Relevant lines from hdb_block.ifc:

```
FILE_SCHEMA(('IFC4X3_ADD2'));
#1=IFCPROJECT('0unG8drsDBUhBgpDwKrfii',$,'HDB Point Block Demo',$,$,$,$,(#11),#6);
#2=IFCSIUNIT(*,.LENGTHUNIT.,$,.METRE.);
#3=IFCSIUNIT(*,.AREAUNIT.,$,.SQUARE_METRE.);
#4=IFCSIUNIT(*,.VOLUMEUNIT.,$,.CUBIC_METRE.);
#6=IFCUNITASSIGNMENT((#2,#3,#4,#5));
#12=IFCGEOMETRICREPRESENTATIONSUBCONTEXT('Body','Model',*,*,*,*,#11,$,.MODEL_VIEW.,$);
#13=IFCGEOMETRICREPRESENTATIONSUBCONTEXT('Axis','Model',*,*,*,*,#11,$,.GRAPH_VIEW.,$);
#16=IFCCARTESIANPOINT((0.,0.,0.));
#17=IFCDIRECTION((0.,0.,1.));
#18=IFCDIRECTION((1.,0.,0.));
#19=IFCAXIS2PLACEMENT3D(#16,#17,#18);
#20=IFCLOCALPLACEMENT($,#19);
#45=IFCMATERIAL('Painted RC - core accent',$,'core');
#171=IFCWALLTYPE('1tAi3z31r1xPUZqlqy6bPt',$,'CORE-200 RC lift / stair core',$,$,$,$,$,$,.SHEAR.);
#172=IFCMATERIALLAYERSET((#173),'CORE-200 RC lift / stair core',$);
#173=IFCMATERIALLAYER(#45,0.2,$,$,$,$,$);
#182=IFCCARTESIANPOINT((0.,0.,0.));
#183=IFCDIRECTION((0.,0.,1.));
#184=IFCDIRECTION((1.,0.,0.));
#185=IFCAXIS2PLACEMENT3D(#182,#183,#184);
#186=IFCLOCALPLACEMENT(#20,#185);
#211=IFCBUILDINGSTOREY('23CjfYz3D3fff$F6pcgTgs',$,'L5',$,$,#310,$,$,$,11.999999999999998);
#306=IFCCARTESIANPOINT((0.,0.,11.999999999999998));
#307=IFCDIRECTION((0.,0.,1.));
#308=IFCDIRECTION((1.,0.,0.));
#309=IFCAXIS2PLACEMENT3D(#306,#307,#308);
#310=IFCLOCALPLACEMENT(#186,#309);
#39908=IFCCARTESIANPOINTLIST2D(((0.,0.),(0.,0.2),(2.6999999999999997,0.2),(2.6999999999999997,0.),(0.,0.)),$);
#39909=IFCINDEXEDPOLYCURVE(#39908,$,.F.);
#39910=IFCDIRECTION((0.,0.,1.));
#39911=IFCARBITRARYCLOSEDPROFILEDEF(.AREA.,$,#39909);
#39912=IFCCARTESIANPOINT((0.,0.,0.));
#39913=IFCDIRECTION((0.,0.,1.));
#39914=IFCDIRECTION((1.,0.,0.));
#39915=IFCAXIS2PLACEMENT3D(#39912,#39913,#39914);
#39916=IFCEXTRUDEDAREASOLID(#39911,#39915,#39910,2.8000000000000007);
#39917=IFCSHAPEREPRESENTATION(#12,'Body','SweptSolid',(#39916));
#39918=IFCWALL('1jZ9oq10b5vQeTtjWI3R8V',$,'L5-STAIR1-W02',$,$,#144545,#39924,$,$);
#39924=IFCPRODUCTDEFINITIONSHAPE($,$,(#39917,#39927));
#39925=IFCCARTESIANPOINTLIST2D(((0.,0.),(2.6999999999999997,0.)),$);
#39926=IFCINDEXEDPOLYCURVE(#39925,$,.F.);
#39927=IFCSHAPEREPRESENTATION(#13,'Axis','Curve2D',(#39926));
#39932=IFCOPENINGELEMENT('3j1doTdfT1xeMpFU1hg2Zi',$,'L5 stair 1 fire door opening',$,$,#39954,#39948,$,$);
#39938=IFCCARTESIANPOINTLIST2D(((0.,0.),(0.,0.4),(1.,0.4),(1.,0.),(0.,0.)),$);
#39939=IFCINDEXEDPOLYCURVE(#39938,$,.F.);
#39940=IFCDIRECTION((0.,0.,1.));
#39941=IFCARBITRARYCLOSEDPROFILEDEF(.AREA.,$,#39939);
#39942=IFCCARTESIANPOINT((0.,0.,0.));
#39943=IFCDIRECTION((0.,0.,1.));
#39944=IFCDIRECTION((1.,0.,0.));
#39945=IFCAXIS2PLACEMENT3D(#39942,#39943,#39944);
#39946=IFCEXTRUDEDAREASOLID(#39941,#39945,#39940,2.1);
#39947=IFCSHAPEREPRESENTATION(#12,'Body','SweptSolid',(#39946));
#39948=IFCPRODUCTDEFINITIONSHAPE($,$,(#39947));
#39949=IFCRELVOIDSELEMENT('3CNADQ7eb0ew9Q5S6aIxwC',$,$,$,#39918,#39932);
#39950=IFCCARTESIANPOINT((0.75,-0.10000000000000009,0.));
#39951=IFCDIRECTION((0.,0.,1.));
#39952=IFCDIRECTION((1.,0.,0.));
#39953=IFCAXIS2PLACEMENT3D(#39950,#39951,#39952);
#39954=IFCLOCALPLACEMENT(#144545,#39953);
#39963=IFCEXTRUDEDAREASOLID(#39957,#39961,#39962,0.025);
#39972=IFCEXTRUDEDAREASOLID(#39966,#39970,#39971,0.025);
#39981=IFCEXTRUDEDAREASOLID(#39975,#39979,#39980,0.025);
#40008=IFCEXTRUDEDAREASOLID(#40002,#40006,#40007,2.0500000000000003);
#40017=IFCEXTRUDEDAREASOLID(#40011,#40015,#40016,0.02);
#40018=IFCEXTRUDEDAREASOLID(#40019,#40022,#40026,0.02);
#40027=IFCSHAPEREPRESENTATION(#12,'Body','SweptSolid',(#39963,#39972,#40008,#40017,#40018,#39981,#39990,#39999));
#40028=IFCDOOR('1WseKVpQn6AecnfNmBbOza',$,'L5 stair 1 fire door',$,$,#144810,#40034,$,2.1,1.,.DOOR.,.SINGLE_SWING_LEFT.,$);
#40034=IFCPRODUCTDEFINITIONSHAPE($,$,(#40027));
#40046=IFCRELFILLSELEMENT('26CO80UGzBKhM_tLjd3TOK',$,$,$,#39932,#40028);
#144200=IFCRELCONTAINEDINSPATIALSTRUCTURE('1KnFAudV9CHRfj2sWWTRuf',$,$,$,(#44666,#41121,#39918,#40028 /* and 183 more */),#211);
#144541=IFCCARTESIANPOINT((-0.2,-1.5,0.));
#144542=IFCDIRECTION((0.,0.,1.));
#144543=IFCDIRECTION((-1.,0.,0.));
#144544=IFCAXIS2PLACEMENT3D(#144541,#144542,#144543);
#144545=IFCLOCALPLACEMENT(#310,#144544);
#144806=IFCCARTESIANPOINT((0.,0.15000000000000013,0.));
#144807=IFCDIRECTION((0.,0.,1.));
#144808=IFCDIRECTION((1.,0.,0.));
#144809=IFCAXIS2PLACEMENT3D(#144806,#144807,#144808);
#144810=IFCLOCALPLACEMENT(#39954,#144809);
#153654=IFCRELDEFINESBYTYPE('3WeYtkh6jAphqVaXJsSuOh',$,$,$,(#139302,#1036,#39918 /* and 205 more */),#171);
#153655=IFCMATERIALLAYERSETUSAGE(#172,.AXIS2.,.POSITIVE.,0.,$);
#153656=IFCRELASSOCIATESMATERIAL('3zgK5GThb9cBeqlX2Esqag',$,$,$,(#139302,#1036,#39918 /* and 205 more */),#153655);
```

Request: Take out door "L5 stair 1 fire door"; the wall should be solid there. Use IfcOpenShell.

```python
import ifcopenshell
import ifcopenshell.api.feature
import ifcopenshell.api.root
import ifcopenshell.geom
import ifcopenshell.util.shape

model = ifcopenshell.open("hdb_block.ifc")
settings = ifcopenshell.geom.settings()


def volume(element):
    """Net volume in cubic metres, openings subtracted."""
    shape = ifcopenshell.geom.create_shape(settings, element)
    return ifcopenshell.util.shape.get_volume(shape.geometry)


door = model.by_id(40028)
opening = door.FillsVoids[0].RelatingOpeningElement
wall = opening.VoidsElements[0].RelatingBuildingElement
before = volume(wall)

ifcopenshell.api.root.remove_product(model, product=door)
ifcopenshell.api.feature.remove_feature(model, feature=opening)

after = volume(wall)

print(f"wall volume {before:.3f} -> {after:.3f} m3")

model.write("hdb_block-out.ifc")
```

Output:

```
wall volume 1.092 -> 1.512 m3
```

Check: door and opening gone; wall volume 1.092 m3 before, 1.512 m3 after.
